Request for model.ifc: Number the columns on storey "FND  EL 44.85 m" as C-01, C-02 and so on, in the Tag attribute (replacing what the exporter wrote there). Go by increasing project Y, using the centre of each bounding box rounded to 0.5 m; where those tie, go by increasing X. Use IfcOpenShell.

First a look at what the model holds.

```python
import ifcopenshell
import ifcopenshell.util.element
import ifcopenshell.util.placement

model = ifcopenshell.open("model.ifc")
print(model.schema)
storey = next(s for s in model.by_type("IfcBuildingStorey") if s.Name == "FND  EL 44.85 m")
columns = [e for e in ifcopenshell.util.element.get_decomposition(storey) if e.is_a("IfcColumn")]
for e in sorted(columns, key=lambda e: e.id()):
    origin = ifcopenshell.util.placement.get_local_placement(e.ObjectPlacement)[:3, 3]
    print(e.id(), e.Tag, e.Name, origin.round(2) + 0.0, sep=" | ")
```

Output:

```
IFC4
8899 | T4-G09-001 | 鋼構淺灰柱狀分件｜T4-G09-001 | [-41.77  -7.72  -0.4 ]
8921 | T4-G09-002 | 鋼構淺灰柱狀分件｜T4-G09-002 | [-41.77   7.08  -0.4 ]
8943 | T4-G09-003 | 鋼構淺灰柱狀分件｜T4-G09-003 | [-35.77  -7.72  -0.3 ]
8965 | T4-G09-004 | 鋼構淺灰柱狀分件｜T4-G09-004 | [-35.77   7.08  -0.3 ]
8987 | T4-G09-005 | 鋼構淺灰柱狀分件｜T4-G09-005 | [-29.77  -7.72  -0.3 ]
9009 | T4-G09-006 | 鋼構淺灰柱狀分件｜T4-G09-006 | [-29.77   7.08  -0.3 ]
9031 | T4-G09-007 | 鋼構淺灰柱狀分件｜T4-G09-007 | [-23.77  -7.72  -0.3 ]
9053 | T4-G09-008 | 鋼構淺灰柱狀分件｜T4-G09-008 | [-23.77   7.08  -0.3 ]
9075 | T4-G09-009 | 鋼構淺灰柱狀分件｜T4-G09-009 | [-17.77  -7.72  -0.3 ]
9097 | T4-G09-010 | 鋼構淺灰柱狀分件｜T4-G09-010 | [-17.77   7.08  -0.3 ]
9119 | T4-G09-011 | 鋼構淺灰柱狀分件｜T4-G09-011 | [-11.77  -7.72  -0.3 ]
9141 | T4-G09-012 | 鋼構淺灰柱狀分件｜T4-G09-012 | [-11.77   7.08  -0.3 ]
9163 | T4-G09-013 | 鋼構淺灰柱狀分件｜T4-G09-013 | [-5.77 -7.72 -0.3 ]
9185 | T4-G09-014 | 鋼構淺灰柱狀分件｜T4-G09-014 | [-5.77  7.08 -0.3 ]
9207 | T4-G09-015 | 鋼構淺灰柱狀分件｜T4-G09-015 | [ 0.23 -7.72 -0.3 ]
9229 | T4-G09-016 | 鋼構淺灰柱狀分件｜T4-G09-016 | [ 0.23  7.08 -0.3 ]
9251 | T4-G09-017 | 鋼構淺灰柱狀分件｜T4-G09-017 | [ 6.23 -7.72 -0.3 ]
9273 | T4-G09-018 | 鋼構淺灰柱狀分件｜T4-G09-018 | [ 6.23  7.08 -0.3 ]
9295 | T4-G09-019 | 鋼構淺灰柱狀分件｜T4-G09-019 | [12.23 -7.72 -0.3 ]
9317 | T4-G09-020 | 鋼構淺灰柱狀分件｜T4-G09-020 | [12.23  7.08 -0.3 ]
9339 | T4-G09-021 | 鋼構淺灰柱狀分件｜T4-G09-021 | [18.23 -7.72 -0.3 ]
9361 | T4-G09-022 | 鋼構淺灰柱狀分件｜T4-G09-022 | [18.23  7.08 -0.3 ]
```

```python
import ifcopenshell
import ifcopenshell.geom
import ifcopenshell.util.element
import ifcopenshell.util.shape

model = ifcopenshell.open("model.ifc")
settings = ifcopenshell.geom.settings()
settings.set("use-world-coords", True)


def centre(element):
    shape = ifcopenshell.geom.create_shape(settings, element)
    return ifcopenshell.util.shape.get_bbox_centroid(shape.geometry)


storey = next(s for s in model.by_type("IfcBuildingStorey") if s.Name == "FND  EL 44.85 m")
columns = [e for e in ifcopenshell.util.element.get_decomposition(storey) if e.is_a("IfcColumn")]

# Insertion points can sit at a corner or the storey origin, so sort by the geometry (in metres).
centres = {e: centre(e) for e in columns}
columns.sort(key=lambda e: (round(centres[e][1] / 0.5), centres[e][0]))

for i, e in enumerate(columns, start=1):
    number = f"C-{i:02d}"
    e.Tag = number
    print(e.id(), number)

model.write("model_v2.ifc")
```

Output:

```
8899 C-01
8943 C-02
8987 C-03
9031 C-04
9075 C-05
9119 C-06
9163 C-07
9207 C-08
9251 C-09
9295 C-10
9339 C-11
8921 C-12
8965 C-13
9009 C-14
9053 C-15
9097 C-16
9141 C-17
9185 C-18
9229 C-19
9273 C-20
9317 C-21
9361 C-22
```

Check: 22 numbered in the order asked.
